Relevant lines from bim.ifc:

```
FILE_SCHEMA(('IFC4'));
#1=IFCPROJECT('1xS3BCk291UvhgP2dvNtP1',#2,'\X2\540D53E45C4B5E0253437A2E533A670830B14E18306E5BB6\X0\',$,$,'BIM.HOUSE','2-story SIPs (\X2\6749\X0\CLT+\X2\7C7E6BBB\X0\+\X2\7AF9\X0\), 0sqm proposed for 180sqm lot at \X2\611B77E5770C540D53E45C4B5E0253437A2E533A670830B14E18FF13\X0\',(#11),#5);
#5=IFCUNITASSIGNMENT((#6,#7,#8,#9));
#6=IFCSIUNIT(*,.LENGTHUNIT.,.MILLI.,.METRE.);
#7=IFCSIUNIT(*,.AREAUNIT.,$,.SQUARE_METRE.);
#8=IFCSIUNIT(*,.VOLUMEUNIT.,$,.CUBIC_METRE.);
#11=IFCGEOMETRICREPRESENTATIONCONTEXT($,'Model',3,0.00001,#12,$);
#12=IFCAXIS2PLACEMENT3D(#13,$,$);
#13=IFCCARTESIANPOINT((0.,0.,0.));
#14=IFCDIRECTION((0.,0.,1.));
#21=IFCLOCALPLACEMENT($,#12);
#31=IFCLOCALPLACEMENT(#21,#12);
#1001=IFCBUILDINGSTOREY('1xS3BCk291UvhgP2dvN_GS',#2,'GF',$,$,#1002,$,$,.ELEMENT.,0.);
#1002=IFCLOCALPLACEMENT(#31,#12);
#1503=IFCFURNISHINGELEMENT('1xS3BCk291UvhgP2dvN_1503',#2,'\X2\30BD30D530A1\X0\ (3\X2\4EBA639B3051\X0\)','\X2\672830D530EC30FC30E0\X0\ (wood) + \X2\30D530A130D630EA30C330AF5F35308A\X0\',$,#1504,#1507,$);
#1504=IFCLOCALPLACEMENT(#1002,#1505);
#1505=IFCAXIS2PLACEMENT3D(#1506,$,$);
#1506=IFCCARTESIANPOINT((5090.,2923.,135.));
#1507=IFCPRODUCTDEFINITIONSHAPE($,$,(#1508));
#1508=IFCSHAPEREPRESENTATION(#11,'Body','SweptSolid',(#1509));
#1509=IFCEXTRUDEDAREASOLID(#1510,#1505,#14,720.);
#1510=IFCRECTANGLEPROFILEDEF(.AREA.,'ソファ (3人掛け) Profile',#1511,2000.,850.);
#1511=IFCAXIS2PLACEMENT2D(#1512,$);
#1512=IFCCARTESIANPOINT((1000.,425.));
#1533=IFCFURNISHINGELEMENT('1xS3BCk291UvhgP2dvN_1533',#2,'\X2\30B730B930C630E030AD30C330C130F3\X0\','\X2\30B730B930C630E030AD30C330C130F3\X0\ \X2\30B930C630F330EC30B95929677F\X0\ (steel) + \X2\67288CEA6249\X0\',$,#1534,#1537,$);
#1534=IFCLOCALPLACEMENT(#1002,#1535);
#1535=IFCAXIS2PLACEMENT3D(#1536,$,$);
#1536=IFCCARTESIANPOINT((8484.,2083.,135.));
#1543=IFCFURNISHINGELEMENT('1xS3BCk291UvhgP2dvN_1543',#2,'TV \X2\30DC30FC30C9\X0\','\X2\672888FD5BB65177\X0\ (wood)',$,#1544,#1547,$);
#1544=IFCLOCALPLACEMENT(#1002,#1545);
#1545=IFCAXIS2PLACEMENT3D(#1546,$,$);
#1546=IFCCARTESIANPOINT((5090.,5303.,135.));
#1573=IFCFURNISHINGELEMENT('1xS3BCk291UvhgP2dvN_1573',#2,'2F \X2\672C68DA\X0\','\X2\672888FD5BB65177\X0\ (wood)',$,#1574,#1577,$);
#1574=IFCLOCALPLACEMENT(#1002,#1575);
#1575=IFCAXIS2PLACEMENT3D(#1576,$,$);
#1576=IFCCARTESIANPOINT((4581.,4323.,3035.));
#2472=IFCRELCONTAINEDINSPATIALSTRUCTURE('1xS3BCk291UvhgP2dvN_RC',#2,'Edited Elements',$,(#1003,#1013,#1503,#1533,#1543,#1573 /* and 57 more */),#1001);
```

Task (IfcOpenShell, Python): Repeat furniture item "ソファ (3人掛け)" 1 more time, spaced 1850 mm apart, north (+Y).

```python
import numpy as np
import ifcopenshell
import ifcopenshell.api.geometry
import ifcopenshell.api.root
import ifcopenshell.util.element
import ifcopenshell.util.placement
import ifcopenshell.util.unit

model = ifcopenshell.open("bim.ifc")
unit_scale = ifcopenshell.util.unit.calculate_unit_scale(model)


def reuse_history(source, copy):
    """copy_class also copies each property set's owner history, people and application; keep the originals."""
    for rel in copy.IsDefinedBy:
        if rel.is_a("IfcRelDefinesByProperties") and (history := rel.RelatingPropertyDefinition.OwnerHistory):
            rel.RelatingPropertyDefinition.OwnerHistory = source.OwnerHistory
            ifcopenshell.util.element.remove_deep2(model, history)


source = model.by_id(1503)
base = ifcopenshell.util.placement.get_local_placement(source.ObjectPlacement)
step = np.array([0.0, 1.0, 0.0]) * 1.85 / unit_scale

for i in range(1, 2):
    copy = ifcopenshell.api.root.copy_class(model, product=source)
    copy.Representation = ifcopenshell.util.element.copy_deep(
        model, source.Representation, exclude=["IfcGeometricRepresentationContext", "IfcRepresentationMap"]
    )
    reuse_history(source, copy)
    matrix = base.copy()
    matrix[:3, 3] += i * step
    print("added at", matrix[:3, 3].round(3) + 0.0)
    ifcopenshell.api.geometry.edit_object_placement(model, product=copy, matrix=matrix, is_si=False)

model.write("bim_updated.ifc")
```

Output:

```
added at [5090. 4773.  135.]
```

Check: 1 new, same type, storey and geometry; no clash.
